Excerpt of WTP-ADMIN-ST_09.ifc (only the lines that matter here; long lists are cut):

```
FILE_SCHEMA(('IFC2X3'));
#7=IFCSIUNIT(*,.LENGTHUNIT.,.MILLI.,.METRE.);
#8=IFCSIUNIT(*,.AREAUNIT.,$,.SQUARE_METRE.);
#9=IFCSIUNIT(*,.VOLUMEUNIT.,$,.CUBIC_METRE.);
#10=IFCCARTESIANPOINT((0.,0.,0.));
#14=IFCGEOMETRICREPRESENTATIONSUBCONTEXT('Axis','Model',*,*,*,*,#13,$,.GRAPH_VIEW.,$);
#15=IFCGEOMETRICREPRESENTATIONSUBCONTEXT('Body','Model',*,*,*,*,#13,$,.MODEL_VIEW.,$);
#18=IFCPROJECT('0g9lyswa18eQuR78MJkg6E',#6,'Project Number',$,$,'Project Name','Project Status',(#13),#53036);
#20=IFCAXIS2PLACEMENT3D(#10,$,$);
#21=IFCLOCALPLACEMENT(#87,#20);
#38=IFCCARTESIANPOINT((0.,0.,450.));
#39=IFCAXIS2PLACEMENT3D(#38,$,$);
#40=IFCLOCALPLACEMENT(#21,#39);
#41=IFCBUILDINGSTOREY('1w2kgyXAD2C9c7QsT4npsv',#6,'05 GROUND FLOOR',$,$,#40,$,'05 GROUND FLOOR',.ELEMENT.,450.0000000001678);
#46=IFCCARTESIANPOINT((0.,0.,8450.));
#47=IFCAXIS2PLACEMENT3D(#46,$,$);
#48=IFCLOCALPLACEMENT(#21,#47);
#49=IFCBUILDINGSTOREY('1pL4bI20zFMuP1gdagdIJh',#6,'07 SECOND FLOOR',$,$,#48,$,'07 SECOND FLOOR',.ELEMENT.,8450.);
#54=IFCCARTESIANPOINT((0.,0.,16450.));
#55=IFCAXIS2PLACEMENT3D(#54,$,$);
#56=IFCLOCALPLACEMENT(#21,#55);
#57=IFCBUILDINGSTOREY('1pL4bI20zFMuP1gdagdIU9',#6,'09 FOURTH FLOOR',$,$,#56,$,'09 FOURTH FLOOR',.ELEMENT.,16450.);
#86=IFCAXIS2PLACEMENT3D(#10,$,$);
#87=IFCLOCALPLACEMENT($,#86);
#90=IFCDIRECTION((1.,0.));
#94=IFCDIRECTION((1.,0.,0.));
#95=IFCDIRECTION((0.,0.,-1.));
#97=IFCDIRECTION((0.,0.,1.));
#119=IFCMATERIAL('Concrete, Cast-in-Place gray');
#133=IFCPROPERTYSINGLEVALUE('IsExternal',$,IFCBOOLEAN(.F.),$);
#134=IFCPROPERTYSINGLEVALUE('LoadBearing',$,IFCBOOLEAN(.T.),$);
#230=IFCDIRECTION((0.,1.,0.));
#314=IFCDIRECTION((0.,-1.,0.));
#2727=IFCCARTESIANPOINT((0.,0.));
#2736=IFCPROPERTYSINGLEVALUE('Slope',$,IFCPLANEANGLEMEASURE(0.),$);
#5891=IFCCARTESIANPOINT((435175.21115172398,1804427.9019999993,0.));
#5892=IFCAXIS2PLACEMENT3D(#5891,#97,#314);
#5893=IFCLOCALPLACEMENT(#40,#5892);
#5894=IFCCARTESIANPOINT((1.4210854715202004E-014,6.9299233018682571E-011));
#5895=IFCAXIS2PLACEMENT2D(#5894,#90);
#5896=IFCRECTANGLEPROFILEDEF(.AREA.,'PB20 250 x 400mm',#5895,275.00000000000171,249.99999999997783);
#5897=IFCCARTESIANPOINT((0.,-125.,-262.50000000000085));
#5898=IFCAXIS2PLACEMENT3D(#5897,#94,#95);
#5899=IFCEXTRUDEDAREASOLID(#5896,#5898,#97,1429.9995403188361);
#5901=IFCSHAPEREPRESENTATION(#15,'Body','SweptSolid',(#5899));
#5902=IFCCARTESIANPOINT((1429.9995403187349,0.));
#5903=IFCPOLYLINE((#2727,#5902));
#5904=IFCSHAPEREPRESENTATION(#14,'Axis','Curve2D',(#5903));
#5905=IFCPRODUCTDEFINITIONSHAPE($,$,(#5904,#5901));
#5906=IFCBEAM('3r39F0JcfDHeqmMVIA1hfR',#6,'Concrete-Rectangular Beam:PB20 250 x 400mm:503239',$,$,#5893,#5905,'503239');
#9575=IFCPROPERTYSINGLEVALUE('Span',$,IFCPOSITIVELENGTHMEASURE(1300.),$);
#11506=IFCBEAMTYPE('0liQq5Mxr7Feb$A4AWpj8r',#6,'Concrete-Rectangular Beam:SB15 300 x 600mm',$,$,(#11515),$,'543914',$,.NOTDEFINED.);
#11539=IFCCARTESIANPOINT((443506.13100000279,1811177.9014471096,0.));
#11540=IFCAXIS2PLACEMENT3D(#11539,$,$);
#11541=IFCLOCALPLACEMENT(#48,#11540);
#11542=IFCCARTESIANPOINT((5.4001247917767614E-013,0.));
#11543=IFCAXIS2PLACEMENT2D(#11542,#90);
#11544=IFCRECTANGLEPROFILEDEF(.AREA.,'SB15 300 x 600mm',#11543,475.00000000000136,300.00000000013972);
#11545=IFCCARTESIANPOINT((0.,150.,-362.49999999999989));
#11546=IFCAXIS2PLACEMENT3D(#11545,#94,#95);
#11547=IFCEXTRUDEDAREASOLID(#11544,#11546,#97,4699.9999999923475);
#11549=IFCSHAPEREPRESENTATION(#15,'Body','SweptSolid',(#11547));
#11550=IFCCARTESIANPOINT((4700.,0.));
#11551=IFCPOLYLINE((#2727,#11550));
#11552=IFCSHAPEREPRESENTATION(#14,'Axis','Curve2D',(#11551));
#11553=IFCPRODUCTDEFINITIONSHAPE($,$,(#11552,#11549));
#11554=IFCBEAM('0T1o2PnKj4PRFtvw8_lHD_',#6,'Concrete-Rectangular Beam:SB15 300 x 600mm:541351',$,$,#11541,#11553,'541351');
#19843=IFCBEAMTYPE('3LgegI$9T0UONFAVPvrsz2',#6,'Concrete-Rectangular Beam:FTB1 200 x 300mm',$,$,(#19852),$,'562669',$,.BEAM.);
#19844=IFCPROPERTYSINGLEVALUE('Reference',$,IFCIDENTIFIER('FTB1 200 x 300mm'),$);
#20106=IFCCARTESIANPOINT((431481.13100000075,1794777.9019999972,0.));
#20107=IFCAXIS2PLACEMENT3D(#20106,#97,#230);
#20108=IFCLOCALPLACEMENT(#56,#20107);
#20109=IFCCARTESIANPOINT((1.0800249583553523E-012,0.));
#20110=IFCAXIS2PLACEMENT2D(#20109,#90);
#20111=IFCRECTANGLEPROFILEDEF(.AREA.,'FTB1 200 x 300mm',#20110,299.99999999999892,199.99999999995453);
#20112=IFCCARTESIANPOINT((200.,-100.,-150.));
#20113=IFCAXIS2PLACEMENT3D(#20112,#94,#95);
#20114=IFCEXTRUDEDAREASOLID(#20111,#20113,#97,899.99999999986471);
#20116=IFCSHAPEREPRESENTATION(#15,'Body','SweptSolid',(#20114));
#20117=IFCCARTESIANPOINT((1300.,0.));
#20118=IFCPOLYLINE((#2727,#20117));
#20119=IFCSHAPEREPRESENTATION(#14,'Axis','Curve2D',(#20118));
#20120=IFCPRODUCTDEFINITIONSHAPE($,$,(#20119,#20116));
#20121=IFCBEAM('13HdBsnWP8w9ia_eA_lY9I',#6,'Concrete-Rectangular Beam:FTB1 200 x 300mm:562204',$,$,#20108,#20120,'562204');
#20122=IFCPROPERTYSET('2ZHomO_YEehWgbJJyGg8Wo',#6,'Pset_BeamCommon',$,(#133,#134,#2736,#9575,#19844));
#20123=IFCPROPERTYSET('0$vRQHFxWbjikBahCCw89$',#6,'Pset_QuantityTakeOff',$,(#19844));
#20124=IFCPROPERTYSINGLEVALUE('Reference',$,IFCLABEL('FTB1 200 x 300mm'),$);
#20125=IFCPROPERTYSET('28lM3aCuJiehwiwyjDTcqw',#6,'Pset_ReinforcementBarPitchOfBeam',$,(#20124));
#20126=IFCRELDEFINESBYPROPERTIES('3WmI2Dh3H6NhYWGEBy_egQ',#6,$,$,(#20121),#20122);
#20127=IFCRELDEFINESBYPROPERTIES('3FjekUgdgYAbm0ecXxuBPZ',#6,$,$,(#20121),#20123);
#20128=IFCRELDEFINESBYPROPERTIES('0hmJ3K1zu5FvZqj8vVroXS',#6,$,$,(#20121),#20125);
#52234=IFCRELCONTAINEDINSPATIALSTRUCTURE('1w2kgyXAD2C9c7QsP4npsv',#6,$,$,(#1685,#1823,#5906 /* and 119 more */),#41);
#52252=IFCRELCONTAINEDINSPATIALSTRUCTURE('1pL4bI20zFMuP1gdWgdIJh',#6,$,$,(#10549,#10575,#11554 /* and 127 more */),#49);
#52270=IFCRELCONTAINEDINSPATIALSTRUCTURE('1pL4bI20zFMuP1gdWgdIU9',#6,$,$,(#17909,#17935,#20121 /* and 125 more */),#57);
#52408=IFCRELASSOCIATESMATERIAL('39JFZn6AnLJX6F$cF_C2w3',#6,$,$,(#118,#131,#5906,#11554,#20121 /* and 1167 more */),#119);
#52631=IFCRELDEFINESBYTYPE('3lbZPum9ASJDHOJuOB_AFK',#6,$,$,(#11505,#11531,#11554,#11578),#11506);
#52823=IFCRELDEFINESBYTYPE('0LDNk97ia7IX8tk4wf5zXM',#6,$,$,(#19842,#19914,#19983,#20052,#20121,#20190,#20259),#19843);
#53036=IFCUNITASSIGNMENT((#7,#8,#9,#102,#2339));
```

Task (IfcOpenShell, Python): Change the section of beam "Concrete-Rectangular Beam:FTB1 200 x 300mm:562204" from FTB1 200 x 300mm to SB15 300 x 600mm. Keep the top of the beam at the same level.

```python
import ifcopenshell
import ifcopenshell.api.pset
import ifcopenshell.api.type
import ifcopenshell.util.element
import ifcopenshell.util.representation

model = ifcopenshell.open("WTP-ADMIN-ST_09.ifc")

member = model.by_guid("13HdBsnWP8w9ia_eA_lY9I")
source = next(p for p in model.by_type("IfcRectangleProfileDef") if p.ProfileName == "SB15 300 x 600mm")

body = ifcopenshell.util.representation.get_representation(member, "Model", "Body")
solid = body.Items[0]
old_profile = solid.SweptArea

# Copy the section's sizes but keep this member's own profile position.
profile = ifcopenshell.util.element.copy(model, source)
# Profiles are centred, so shift by half the change in depth to hold the top.
shift = (old_profile.XDim - profile.XDim) / 2
x, y = old_profile.Position.Location.Coordinates
up = (-1.0, 0.0)  # upwards, in the solid's own plane
location = model.createIfcCartesianPoint((x + up[0] * shift, y + up[1] * shift))
profile.Position = model.createIfcAxis2Placement2D(location, old_profile.Position.RefDirection)
solid.SweptArea = profile
if not model.get_total_inverses(old_profile):
    ifcopenshell.util.element.remove_deep2(model, old_profile)

new_type = model.by_guid("0liQq5Mxr7Feb$A4AWpj8r")
ifcopenshell.api.type.assign_type(
    model, related_objects=[member], relating_type=new_type, should_map_representations=False
)
member.Name = member.Name.replace("FTB1 200 x 300mm", "SB15 300 x 600mm")
pset = model.by_id(ifcopenshell.util.element.get_pset(member, "Pset_BeamCommon", should_inherit=False)["id"])
ifcopenshell.api.pset.edit_pset(model, pset=pset, properties={"Reference": "SB15 300 x 600mm"})
pset = model.by_id(ifcopenshell.util.element.get_pset(member, "Pset_QuantityTakeOff", should_inherit=False)["id"])
ifcopenshell.api.pset.edit_pset(model, pset=pset, properties={"Reference": "SB15 300 x 600mm"})
pset = model.by_id(ifcopenshell.util.element.get_pset(member, "Pset_ReinforcementBarPitchOfBeam", should_inherit=False)["id"])
ifcopenshell.api.pset.edit_pset(model, pset=pset, properties={"Reference": "SB15 300 x 600mm"})

print(solid.SweptArea)

model.write("WTP-ADMIN-ST_09_updated.ifc")
```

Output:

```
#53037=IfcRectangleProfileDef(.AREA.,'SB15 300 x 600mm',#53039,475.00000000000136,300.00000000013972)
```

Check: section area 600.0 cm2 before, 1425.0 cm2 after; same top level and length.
